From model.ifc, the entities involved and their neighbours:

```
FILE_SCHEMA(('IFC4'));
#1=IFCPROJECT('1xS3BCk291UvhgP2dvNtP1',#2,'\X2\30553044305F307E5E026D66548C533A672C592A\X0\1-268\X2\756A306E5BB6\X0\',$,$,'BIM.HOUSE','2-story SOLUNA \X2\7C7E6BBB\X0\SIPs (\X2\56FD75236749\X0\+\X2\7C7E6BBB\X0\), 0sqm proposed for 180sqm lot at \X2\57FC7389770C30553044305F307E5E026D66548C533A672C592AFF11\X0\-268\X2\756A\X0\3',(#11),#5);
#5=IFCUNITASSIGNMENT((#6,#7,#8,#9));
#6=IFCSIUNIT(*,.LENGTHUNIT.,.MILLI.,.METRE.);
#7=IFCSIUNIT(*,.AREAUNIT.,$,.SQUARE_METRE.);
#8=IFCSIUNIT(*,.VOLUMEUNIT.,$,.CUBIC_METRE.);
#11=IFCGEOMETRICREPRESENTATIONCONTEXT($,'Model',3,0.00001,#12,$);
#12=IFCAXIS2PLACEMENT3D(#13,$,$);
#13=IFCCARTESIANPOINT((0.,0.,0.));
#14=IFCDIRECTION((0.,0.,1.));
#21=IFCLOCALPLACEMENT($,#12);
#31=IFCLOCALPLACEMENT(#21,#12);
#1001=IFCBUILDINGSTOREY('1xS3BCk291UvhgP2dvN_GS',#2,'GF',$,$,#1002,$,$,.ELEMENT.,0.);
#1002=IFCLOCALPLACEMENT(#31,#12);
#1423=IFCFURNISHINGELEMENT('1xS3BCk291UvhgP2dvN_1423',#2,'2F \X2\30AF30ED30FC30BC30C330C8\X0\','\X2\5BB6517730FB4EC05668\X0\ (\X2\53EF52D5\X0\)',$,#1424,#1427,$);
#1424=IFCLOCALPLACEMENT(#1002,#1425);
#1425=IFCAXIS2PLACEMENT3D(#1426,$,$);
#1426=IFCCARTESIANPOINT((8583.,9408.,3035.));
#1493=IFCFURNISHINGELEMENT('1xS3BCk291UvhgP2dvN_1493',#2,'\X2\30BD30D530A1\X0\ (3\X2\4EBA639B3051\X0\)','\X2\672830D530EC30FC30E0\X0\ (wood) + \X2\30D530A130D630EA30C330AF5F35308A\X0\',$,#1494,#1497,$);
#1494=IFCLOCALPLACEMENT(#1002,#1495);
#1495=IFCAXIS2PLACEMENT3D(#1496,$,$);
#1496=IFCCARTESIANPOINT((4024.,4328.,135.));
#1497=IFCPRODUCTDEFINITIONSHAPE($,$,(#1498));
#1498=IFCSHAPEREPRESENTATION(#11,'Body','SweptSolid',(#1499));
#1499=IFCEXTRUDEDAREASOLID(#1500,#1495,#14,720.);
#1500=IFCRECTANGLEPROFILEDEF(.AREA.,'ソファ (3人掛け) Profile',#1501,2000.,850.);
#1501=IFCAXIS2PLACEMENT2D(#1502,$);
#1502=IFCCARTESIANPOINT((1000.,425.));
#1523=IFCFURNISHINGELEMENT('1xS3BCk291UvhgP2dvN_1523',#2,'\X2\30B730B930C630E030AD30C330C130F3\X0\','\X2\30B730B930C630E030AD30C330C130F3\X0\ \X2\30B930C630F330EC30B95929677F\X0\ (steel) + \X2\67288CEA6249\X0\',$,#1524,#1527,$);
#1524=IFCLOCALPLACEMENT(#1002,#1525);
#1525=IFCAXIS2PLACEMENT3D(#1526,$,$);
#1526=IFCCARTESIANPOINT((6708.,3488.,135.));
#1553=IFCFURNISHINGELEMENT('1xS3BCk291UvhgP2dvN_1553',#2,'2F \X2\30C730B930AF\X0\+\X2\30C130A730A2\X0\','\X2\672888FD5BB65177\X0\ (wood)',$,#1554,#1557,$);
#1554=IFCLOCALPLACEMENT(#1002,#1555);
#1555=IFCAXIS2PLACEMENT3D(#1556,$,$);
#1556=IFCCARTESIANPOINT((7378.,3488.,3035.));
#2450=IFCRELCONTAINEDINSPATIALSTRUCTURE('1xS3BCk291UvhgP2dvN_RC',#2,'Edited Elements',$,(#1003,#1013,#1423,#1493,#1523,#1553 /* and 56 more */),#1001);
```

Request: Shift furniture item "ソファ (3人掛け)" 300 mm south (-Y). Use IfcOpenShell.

```python
import ifcopenshell
import ifcopenshell.api.geometry
import ifcopenshell.util.placement
import ifcopenshell.util.unit

model = ifcopenshell.open("model.ifc")
unit_scale = ifcopenshell.util.unit.calculate_unit_scale(model)

item = model.by_guid("1xS3BCk291UvhgP2dvN_1493")
matrix = ifcopenshell.util.placement.get_local_placement(item.ObjectPlacement)
matrix[1, 3] -= 0.3 / unit_scale
ifcopenshell.api.geometry.edit_object_placement(model, product=item, matrix=matrix, is_si=False)

print(ifcopenshell.util.placement.get_local_placement(item.ObjectPlacement).round(3) + 0.0)

model.write("model_v2.ifc")
```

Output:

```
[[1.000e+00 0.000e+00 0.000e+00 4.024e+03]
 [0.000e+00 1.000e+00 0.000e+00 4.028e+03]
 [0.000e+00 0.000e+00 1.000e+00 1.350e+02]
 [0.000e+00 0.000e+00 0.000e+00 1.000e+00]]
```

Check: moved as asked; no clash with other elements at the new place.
